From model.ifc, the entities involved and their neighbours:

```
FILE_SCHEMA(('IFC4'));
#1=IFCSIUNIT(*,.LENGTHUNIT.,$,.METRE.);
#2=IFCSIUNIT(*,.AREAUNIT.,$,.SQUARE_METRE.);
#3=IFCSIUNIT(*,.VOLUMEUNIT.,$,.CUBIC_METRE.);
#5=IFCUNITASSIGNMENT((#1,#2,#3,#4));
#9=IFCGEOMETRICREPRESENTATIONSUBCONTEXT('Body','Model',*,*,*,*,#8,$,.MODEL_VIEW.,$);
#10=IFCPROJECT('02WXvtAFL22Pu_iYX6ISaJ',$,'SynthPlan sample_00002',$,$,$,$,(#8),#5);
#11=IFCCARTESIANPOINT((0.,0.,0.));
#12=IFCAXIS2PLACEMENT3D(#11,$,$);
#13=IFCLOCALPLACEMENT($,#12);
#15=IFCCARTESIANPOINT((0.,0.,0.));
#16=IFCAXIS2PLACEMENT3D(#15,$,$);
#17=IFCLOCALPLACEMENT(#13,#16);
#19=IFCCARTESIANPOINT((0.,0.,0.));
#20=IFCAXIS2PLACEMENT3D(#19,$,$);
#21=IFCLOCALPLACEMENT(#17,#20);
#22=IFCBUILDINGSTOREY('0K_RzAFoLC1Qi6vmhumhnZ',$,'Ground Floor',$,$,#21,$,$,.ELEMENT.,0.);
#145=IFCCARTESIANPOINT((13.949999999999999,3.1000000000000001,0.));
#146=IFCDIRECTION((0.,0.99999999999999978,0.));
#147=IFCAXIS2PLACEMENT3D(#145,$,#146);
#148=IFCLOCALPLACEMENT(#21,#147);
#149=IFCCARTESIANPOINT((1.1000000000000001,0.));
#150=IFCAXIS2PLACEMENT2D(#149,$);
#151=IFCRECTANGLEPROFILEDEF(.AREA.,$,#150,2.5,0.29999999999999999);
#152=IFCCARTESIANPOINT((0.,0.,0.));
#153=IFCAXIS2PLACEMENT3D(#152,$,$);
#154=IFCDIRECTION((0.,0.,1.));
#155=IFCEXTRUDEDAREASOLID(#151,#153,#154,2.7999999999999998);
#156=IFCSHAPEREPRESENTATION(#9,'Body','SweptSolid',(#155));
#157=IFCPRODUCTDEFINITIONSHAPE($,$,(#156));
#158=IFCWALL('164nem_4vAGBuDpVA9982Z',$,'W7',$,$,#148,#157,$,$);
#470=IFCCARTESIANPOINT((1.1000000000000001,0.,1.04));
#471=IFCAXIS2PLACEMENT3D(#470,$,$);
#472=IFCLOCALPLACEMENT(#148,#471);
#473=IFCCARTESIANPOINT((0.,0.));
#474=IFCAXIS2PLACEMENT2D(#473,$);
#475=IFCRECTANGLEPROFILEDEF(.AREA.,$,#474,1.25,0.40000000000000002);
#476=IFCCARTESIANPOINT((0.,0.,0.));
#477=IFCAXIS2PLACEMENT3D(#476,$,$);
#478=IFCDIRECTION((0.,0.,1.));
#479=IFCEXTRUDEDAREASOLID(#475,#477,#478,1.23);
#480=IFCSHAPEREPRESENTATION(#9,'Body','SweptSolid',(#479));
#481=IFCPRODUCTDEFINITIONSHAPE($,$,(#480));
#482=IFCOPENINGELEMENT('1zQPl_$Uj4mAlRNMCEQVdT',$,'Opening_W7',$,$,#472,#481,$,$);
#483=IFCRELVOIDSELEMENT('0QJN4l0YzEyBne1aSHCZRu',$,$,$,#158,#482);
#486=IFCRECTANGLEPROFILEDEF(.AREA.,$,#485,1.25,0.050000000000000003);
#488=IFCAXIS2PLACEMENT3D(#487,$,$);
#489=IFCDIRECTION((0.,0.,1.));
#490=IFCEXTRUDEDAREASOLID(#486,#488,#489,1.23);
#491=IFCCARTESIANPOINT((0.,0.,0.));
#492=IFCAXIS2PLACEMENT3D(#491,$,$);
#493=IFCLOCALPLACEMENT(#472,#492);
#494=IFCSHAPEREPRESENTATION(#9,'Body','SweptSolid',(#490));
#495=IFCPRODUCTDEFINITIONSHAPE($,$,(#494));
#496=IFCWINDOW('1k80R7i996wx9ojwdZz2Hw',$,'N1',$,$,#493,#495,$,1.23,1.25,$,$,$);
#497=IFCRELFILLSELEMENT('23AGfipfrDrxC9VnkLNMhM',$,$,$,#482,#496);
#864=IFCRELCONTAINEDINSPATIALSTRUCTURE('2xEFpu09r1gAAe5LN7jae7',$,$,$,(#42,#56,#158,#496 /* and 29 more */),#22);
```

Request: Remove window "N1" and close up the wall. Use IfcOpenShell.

```python
import ifcopenshell
import ifcopenshell.api.feature
import ifcopenshell.api.root
import ifcopenshell.geom
import ifcopenshell.util.shape

model = ifcopenshell.open("model.ifc")
settings = ifcopenshell.geom.settings()


def volume(element):
    """Net volume in cubic metres, openings subtracted."""
    shape = ifcopenshell.geom.create_shape(settings, element)
    return ifcopenshell.util.shape.get_volume(shape.geometry)


window = model.by_guid("1k80R7i996wx9ojwdZz2Hw")
opening = window.FillsVoids[0].RelatingOpeningElement
wall = opening.VoidsElements[0].RelatingBuildingElement
before = volume(wall)

ifcopenshell.api.root.remove_product(model, product=window)
ifcopenshell.api.feature.remove_feature(model, feature=opening)

after = volume(wall)

print(f"wall volume {before:.3f} -> {after:.3f} m3")

model.write("model_edited.ifc")
```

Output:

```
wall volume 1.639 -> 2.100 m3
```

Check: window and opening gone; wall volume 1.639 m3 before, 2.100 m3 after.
